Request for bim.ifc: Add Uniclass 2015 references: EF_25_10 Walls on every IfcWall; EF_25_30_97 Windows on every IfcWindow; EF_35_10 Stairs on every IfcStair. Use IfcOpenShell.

First a look at what the model holds.

```python
import ifcopenshell

model = ifcopenshell.open("bim.ifc")
print(model.schema)
print("classifications:", [c.Name for c in model.by_type("IfcClassification")])
for ifc_class in ("IfcDoor", "IfcRoof", "IfcStair", "IfcWall", "IfcWindow"):
    print(ifc_class, len(model.by_type(ifc_class)))
```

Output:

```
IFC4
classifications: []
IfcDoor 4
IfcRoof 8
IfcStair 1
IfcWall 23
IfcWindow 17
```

```python
import ifcopenshell
import ifcopenshell.api.classification

model = ifcopenshell.open("bim.ifc")

system = ifcopenshell.api.classification.add_classification(model, classification="Uniclass 2015")

codes = {
    "IfcWall": ("EF_25_10", "Walls"),
    "IfcWindow": ("EF_25_30_97", "Windows"),
    "IfcStair": ("EF_35_10", "Stairs"),
}
for ifc_class, (code, name) in codes.items():
    products = model.by_type(ifc_class)
    ifcopenshell.api.classification.add_reference(
        model, products=products, classification=system, identification=code, name=name
    )
    print(code, len(products))

model.write("bim_rev.ifc")
```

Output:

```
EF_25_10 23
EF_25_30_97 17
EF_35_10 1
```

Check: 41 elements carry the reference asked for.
